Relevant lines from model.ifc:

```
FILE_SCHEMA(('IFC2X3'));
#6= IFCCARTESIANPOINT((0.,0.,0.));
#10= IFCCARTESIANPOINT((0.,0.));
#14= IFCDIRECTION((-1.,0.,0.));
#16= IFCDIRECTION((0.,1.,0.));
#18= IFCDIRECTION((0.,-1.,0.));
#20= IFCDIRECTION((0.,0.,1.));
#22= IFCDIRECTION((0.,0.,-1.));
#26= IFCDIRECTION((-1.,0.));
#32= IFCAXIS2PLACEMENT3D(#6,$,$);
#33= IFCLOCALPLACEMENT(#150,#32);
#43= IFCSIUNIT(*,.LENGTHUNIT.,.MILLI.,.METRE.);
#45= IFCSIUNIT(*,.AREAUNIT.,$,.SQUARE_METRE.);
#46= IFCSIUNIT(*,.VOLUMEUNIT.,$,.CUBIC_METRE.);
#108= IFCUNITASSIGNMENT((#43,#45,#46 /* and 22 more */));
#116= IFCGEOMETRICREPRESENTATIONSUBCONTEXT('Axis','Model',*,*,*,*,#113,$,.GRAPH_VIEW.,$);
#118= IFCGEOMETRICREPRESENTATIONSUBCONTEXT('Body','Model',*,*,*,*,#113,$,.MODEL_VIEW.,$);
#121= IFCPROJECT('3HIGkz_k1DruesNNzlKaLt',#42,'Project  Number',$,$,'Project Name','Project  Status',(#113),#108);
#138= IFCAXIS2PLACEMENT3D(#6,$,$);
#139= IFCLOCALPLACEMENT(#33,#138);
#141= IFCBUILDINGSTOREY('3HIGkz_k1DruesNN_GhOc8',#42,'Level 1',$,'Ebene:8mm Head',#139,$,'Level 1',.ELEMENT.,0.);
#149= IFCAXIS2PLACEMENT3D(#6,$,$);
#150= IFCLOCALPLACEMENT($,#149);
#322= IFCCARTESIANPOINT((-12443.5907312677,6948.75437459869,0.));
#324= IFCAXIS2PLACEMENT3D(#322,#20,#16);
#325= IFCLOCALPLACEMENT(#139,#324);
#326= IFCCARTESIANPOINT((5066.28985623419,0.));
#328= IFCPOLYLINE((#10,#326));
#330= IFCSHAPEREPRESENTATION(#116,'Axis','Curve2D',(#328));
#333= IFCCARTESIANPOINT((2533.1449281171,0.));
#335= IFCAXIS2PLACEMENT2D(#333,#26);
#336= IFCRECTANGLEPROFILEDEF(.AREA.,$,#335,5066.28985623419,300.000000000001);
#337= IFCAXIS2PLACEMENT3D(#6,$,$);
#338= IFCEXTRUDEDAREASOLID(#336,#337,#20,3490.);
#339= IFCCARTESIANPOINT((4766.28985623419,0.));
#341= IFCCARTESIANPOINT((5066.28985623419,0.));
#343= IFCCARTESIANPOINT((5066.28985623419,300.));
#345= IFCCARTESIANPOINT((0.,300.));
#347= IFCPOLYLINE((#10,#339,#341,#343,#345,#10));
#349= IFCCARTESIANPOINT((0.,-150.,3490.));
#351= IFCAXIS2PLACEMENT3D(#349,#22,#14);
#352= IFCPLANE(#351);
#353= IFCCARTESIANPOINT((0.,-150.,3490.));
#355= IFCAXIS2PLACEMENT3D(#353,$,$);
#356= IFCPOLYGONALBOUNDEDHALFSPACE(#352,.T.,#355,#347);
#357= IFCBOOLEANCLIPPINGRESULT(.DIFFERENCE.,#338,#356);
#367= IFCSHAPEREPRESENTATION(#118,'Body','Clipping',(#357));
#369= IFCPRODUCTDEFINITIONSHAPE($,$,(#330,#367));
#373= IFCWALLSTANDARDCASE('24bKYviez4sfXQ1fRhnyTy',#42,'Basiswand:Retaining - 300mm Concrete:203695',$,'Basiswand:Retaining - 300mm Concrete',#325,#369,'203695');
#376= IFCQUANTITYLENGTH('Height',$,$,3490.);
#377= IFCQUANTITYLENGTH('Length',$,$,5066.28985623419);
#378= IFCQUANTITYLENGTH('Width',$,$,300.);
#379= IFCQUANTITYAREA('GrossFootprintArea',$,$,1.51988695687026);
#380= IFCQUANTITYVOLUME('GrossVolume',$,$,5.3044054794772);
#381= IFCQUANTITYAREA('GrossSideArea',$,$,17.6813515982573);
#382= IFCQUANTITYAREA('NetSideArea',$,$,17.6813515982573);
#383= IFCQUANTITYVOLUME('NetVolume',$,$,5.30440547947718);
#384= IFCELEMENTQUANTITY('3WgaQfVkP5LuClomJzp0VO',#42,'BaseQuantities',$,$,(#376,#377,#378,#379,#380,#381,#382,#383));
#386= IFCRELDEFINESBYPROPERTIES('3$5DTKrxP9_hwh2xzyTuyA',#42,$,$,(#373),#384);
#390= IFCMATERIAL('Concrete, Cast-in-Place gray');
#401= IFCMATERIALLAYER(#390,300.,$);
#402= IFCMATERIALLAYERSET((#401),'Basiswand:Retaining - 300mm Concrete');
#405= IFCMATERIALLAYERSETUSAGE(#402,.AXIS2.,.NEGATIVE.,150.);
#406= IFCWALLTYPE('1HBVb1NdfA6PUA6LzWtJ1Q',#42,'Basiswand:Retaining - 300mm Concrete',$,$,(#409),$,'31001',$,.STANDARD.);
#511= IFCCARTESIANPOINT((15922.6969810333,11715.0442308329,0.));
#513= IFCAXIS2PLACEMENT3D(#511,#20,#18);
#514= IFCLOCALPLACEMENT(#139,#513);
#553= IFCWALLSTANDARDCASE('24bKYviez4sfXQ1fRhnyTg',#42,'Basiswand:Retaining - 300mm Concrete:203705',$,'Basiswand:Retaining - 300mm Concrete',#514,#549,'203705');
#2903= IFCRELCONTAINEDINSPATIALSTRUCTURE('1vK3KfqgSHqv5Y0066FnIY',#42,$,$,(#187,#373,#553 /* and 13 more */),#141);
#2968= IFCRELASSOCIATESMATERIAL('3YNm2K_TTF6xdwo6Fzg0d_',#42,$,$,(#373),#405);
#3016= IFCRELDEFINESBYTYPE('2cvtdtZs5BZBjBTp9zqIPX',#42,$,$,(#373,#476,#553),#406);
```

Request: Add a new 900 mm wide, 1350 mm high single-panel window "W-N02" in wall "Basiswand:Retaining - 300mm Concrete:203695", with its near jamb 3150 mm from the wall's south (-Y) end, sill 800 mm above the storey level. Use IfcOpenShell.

```python
import numpy as np
import ifcopenshell
import ifcopenshell.api.feature
import ifcopenshell.api.geometry
import ifcopenshell.api.pset
import ifcopenshell.api.root
import ifcopenshell.api.spatial
import ifcopenshell.api.type
import ifcopenshell.geom
import ifcopenshell.util.element
import ifcopenshell.util.placement
import ifcopenshell.util.representation
import ifcopenshell.util.shape
import ifcopenshell.util.unit

model = ifcopenshell.open("model.ifc")
unit_scale = ifcopenshell.util.unit.calculate_unit_scale(model)
area_scale = ifcopenshell.util.unit.calculate_unit_scale(model, "AREAUNIT")
volume_scale = ifcopenshell.util.unit.calculate_unit_scale(model, "VOLUMEUNIT")
settings = ifcopenshell.geom.settings()


def volume(element):
    """Net volume in cubic metres, openings subtracted."""
    shape = ifcopenshell.geom.create_shape(settings, element)
    return ifcopenshell.util.shape.get_volume(shape.geometry)


wall = model.by_guid("24bKYviez4sfXQ1fRhnyTy")
storey = ifcopenshell.util.element.get_container(wall, ifc_class="IfcBuildingStorey")
context = ifcopenshell.util.representation.get_context(model, "Model", "Body", "MODEL_VIEW")
before = volume(wall)

width, height, from_end, sill = 0.9, 1.35, 3.15, 0.8  # metres

# The wall runs along its own X axis, and the end named is its -X end.
wall_shape = ifcopenshell.geom.create_shape(settings, wall)
x, y, z = ifcopenshell.util.shape.get_vertices(wall_shape.geometry).T
start = x.min() + from_end
face, thickness = float(y.min()), float(y.max() - y.min())
wall_matrix = ifcopenshell.util.placement.get_local_placement(wall.ObjectPlacement)
level = ifcopenshell.util.placement.get_local_placement(storey.ObjectPlacement)[2, 3]


def in_wall(x, y):
    """Placement at x, y metres in the wall's axes, at sill height."""
    matrix = wall_matrix.copy()
    matrix[:, 3] = wall_matrix @ np.array([x / unit_scale, y / unit_scale, 0.0, 1.0])
    matrix[2, 3] = level + sill / unit_scale
    return matrix


# Opening: a box that overshoots both wall faces by 50 mm.
opening = ifcopenshell.api.root.create_entity(model, ifc_class="IfcOpeningElement")
box = ifcopenshell.api.geometry.add_wall_representation(
    model, context=context, length=width, height=height, thickness=thickness + 0.1
)
ifcopenshell.api.geometry.assign_representation(model, product=opening, representation=box)
ifcopenshell.api.geometry.edit_object_placement(model, product=opening, matrix=in_wall(start, face - 0.05), is_si=False)
ifcopenshell.api.feature.add_feature(model, feature=opening, element=wall)

window = ifcopenshell.api.root.create_entity(model, ifc_class="IfcWindow", name="W-N02")
window.OverallWidth, window.OverallHeight = width / unit_scale, height / unit_scale
body = ifcopenshell.api.geometry.add_window_representation(
    model,
    context=context,
    overall_width=window.OverallWidth,
    overall_height=window.OverallHeight,
    partition_type="SINGLE_PANEL",
)
ifcopenshell.api.geometry.assign_representation(model, product=window, representation=body)
ifcopenshell.api.spatial.assign_container(model, products=[window], relating_structure=storey)
fills = ifcopenshell.api.feature.add_filling(model, opening=opening, element=window)
fills.OwnerHistory = window.OwnerHistory  # required in IFC2X3

# IFC2X3 keeps the operation on the window style.
style = ifcopenshell.api.root.create_entity(model, ifc_class="IfcWindowStyle", name="W-N02")
style.OperationType, style.ConstructionType = "SINGLE_PANEL", "NOTDEFINED"
style.ParameterTakesPrecedence = style.Sizeable = False
ifcopenshell.api.type.assign_type(model, related_objects=[window], relating_type=style)

# Centre the window in the wall's thickness.
ifcopenshell.api.geometry.edit_object_placement(model, product=window, matrix=in_wall(start, face), is_si=False)
window_shape = ifcopenshell.geom.create_shape(settings, window)
depth = ifcopenshell.util.shape.get_vertices(window_shape.geometry)[:, 1]
offset = face + thickness / 2 - (depth.min() + depth.max()) / 2
ifcopenshell.api.geometry.edit_object_placement(model, product=window, matrix=in_wall(start, offset), is_si=False)

after = volume(wall)

# Update the wall's stored quantities.
qto = model.by_id(ifcopenshell.util.element.get_pset(wall, "BaseQuantities", should_inherit=False)["id"])
ifcopenshell.api.pset.edit_qto(model, qto=qto, properties={
    "NetSideArea": after / thickness / area_scale,
    "NetVolume": after / volume_scale,
})

print(f"wall volume {before:.3f} -> {after:.3f} m3")

model.write("model-out.ifc")
```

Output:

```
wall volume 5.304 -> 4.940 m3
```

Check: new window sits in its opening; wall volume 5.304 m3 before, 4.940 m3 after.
